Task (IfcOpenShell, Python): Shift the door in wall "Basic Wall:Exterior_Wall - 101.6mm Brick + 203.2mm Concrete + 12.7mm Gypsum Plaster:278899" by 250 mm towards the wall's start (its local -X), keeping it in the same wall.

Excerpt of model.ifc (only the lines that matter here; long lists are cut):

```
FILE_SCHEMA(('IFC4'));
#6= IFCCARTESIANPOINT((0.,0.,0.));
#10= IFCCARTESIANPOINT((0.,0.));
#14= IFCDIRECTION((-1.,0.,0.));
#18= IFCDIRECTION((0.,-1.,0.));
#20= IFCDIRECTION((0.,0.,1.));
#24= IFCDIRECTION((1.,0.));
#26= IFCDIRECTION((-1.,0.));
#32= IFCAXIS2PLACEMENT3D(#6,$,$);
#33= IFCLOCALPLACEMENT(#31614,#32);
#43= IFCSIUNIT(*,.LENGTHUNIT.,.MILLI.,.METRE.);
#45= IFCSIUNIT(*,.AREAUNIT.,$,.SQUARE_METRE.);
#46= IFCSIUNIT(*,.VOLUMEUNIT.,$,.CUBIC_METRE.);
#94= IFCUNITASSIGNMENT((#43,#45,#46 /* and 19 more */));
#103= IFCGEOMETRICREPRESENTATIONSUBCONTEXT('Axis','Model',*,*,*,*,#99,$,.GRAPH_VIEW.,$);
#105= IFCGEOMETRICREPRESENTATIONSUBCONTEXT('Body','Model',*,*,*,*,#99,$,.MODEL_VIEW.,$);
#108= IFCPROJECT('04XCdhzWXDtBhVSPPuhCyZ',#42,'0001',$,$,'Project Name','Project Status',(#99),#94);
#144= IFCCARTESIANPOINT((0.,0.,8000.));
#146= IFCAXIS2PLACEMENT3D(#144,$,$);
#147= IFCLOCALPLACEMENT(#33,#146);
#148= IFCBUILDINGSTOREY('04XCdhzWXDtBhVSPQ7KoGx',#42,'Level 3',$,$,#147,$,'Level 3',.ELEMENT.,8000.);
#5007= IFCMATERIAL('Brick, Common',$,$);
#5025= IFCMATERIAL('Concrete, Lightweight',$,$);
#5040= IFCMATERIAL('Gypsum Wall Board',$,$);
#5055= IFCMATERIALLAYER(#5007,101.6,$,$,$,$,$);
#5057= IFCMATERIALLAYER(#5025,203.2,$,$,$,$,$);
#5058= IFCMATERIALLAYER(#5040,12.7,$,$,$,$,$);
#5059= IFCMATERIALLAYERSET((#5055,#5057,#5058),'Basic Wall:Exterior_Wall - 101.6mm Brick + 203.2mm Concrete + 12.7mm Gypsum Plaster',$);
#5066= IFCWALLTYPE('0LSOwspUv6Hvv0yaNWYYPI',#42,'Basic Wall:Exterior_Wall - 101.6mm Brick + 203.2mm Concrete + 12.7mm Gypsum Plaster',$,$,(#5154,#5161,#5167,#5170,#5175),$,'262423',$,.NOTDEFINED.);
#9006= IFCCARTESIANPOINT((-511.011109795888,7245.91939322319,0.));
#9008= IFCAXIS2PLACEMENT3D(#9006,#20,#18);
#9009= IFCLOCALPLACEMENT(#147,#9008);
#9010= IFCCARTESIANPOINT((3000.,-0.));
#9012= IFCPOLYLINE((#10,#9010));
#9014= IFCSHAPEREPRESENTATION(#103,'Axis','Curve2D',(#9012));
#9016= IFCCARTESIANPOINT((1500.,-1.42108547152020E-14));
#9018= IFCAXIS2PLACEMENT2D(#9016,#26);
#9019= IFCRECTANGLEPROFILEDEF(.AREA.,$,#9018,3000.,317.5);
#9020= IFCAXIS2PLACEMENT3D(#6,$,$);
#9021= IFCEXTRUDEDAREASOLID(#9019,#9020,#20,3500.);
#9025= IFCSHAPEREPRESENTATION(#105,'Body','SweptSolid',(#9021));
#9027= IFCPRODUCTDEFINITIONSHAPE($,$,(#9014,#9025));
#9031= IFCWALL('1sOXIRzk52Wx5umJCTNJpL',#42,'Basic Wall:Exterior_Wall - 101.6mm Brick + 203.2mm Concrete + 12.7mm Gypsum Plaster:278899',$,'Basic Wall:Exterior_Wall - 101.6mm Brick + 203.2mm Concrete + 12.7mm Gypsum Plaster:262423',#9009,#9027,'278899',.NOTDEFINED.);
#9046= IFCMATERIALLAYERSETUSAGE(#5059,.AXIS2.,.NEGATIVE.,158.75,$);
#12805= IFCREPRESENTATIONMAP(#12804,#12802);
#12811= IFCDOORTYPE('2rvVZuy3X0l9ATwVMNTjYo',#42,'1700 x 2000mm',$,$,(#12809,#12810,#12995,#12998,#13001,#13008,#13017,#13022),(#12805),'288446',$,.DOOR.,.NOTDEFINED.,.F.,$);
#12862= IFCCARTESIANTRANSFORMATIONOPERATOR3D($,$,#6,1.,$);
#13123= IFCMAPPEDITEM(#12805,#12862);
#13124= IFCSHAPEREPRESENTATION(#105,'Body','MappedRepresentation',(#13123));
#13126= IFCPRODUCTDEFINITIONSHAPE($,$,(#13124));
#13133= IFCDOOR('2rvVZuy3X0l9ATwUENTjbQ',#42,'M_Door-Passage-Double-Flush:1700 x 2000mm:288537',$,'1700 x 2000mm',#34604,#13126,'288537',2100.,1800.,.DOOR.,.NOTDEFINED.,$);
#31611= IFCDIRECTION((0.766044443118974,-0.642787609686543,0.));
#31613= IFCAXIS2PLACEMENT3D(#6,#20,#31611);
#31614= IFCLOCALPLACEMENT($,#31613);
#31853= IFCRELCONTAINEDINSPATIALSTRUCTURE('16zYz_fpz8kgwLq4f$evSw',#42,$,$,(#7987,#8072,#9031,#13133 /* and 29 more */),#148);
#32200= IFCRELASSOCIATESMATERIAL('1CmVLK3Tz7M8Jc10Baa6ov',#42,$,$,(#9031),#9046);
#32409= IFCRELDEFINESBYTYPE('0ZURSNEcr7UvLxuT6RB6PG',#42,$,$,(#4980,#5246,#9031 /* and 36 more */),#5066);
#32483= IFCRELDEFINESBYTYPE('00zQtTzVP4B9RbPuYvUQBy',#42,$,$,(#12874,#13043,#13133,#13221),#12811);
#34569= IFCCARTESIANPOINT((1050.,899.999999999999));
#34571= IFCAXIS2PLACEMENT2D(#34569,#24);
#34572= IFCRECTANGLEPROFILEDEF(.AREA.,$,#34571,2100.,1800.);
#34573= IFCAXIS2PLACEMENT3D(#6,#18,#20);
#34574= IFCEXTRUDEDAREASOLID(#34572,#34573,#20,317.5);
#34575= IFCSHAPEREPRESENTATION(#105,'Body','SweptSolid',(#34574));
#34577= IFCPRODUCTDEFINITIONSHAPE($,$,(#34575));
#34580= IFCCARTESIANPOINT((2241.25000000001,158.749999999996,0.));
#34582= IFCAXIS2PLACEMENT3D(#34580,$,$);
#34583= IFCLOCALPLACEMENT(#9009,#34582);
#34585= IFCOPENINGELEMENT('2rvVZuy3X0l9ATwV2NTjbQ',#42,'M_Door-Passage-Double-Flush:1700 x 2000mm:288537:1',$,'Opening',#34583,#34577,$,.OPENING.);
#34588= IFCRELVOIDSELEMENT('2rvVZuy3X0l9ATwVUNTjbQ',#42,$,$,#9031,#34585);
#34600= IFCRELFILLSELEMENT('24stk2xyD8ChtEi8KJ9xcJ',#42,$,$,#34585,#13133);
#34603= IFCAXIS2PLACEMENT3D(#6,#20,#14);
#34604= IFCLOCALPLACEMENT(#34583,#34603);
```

```python
import ifcopenshell
import ifcopenshell.api.geometry
import ifcopenshell.util.placement
import ifcopenshell.util.unit

model = ifcopenshell.open("model.ifc")
unit_scale = ifcopenshell.util.unit.calculate_unit_scale(model)

door = model.by_guid("2rvVZuy3X0l9ATwUENTjbQ")
opening = door.FillsVoids[0].RelatingOpeningElement
wall = opening.VoidsElements[0].RelatingBuildingElement

wall_matrix = ifcopenshell.util.placement.get_local_placement(wall.ObjectPlacement)
shift = wall_matrix[:3, 0] * -0.25 / unit_scale
before = ifcopenshell.util.placement.get_local_placement(door.ObjectPlacement)[:3, 3].copy()

# The door is placed relative to its opening, so it follows when the opening moves.
matrix = ifcopenshell.util.placement.get_local_placement(opening.ObjectPlacement)
matrix[:3, 3] += shift
ifcopenshell.api.geometry.edit_object_placement(
    model, product=opening, matrix=matrix, is_si=False, should_transform_children=True
)

after = ifcopenshell.util.placement.get_local_placement(door.ObjectPlacement)[:3, 3]
print("door moved by", (after - before).round(3) + 0.0)

model.write("model_updated.ifc")
```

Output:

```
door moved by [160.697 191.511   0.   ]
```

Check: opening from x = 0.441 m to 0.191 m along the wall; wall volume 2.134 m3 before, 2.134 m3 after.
